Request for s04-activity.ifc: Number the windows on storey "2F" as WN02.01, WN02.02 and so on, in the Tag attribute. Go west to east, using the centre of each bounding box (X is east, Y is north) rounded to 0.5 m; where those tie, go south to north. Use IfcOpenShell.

First a look at what the model holds.

```python
import ifcopenshell
import ifcopenshell.util.element
import ifcopenshell.util.placement

model = ifcopenshell.open("s04-activity.ifc")
print(model.schema)
storey = next(s for s in model.by_type("IfcBuildingStorey") if s.Name == "2F")
windows = [e for e in ifcopenshell.util.element.get_decomposition(storey) if e.is_a("IfcWindow")]
for e in sorted(windows, key=lambda e: e.id()):
    origin = ifcopenshell.util.placement.get_local_placement(e.ObjectPlacement)[:3, 3]
    print(e.id(), e.Tag, e.Name, origin.round(2) + 0.0, sep=" | ")
```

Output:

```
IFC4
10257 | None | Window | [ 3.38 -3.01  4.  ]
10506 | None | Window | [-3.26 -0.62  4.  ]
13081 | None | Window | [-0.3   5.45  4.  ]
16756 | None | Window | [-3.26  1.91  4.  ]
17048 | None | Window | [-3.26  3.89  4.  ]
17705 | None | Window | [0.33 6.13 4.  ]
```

```python
import ifcopenshell
import ifcopenshell.geom
import ifcopenshell.util.element
import ifcopenshell.util.shape

model = ifcopenshell.open("s04-activity.ifc")
settings = ifcopenshell.geom.settings()
settings.set("use-world-coords", True)


def centre(element):
    shape = ifcopenshell.geom.create_shape(settings, element)
    return ifcopenshell.util.shape.get_bbox_centroid(shape.geometry)


storey = next(s for s in model.by_type("IfcBuildingStorey") if s.Name == "2F")
windows = [e for e in ifcopenshell.util.element.get_decomposition(storey) if e.is_a("IfcWindow")]

# Insertion points can sit at a corner or the storey origin, so sort by the geometry (in metres).
centres = {e: centre(e) for e in windows}
windows.sort(key=lambda e: (round(centres[e][0] / 0.5), centres[e][1]))

for i, e in enumerate(windows, start=1):
    number = f"WN02.{i:02d}"
    e.Tag = number
    print(e.id(), number)

model.write("s04-activity-out.ifc")
```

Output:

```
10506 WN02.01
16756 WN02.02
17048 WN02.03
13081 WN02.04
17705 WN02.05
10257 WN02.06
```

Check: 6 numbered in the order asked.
